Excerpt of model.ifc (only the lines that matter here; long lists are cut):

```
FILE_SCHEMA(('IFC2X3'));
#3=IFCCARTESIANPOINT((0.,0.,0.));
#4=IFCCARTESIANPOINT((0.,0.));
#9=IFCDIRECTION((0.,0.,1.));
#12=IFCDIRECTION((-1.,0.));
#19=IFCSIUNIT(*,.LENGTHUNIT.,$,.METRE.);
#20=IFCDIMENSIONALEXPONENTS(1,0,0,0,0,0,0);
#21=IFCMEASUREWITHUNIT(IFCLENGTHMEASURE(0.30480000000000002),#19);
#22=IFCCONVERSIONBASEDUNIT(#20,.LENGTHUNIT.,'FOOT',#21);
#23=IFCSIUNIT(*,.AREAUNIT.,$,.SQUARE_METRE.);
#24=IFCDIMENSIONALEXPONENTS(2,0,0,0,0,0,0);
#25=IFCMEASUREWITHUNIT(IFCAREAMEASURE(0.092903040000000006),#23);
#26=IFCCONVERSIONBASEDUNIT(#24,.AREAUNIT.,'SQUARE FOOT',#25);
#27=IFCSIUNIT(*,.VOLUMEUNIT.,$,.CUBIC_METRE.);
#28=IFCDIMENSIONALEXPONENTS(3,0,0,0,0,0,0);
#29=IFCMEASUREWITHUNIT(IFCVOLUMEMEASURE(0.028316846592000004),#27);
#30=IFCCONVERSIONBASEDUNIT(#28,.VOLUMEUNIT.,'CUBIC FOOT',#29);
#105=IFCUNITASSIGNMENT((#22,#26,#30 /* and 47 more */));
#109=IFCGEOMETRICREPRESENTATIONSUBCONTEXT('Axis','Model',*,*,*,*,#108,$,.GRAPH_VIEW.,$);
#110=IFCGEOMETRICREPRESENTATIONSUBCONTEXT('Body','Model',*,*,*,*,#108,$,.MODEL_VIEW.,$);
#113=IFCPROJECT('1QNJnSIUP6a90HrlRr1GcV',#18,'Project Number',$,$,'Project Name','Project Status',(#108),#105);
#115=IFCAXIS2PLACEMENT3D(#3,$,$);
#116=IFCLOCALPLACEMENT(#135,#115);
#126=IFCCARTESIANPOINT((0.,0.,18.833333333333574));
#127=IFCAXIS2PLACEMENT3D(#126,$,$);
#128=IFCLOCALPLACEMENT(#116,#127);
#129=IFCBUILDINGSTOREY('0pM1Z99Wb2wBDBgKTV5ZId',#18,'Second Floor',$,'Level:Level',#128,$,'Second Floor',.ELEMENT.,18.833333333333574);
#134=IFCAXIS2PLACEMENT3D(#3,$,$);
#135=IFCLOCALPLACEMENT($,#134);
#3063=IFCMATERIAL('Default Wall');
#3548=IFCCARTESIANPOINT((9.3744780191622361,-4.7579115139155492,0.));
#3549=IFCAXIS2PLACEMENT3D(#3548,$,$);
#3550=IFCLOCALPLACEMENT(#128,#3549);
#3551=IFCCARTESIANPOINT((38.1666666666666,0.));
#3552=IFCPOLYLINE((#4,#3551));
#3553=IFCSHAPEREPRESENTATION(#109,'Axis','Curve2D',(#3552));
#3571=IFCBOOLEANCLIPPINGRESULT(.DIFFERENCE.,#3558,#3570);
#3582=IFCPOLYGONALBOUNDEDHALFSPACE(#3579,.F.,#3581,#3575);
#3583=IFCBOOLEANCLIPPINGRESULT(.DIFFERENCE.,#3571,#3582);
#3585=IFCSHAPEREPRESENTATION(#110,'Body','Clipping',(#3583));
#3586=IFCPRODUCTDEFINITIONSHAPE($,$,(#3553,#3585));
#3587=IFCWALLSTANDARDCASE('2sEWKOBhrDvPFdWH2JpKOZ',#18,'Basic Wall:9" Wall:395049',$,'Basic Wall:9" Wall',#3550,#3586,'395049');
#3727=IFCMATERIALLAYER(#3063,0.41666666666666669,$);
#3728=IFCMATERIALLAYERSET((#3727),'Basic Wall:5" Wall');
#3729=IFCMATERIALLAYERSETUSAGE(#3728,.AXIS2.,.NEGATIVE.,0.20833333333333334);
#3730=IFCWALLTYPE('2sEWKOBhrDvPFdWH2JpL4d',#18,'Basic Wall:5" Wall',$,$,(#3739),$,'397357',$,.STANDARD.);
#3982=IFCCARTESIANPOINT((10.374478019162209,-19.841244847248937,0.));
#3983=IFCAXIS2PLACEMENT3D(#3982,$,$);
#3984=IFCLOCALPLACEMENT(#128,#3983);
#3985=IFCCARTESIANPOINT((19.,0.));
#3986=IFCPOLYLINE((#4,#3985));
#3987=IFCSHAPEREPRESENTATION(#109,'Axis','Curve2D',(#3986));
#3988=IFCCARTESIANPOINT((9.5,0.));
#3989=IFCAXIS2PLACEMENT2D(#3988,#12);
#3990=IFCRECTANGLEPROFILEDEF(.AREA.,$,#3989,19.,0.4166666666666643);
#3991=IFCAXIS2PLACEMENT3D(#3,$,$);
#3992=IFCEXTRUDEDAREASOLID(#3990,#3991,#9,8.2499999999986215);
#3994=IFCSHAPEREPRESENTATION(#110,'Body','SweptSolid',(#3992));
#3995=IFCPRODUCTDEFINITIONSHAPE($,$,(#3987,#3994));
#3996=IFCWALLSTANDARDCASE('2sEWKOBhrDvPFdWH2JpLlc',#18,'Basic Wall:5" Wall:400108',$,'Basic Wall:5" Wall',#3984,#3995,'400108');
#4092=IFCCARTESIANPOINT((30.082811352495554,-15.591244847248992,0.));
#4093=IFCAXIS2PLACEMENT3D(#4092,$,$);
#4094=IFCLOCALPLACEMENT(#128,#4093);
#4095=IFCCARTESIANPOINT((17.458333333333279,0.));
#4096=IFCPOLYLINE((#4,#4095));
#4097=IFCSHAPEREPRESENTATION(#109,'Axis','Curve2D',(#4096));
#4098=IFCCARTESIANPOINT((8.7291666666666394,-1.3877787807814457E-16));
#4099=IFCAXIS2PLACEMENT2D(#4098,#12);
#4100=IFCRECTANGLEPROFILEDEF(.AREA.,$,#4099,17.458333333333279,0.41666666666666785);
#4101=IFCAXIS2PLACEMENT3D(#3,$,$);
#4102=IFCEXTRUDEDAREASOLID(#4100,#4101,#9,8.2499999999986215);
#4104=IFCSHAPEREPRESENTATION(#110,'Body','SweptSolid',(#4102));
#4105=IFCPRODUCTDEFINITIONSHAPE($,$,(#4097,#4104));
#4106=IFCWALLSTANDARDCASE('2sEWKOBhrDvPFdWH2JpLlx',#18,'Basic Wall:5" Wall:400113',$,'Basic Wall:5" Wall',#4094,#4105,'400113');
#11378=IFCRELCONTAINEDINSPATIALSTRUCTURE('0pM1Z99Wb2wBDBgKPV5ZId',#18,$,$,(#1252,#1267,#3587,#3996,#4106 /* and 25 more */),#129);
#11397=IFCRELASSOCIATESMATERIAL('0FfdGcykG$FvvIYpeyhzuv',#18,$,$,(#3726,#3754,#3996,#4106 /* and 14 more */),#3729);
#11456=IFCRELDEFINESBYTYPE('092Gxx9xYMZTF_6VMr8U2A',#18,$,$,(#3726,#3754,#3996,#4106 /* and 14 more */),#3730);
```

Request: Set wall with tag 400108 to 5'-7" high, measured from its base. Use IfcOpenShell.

```python
import ifcopenshell
import ifcopenshell.geom
import ifcopenshell.util.representation
import ifcopenshell.util.shape
import ifcopenshell.util.unit

model = ifcopenshell.open("model.ifc")
unit_scale = ifcopenshell.util.unit.calculate_unit_scale(model)
settings = ifcopenshell.geom.settings()


def volume(element):
    """Net volume in cubic metres, openings subtracted."""
    shape = ifcopenshell.geom.create_shape(settings, element)
    return ifcopenshell.util.shape.get_volume(shape.geometry)


wall = model.by_guid("2sEWKOBhrDvPFdWH2JpLlc")
before = volume(wall)

body = ifcopenshell.util.representation.get_representation(wall, "Model", "Body")
solid = body.Items[0]
old_height = solid.Depth
solid.Depth = 67 * 0.0254 / unit_scale
after = volume(wall)

print(f"height {old_height:g} -> {solid.Depth:g}, volume {before:.3f} -> {after:.3f} m3")

model.write("model_edited.ifc")
```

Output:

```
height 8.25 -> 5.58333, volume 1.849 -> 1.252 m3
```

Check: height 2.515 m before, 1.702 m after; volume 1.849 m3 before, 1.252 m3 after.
